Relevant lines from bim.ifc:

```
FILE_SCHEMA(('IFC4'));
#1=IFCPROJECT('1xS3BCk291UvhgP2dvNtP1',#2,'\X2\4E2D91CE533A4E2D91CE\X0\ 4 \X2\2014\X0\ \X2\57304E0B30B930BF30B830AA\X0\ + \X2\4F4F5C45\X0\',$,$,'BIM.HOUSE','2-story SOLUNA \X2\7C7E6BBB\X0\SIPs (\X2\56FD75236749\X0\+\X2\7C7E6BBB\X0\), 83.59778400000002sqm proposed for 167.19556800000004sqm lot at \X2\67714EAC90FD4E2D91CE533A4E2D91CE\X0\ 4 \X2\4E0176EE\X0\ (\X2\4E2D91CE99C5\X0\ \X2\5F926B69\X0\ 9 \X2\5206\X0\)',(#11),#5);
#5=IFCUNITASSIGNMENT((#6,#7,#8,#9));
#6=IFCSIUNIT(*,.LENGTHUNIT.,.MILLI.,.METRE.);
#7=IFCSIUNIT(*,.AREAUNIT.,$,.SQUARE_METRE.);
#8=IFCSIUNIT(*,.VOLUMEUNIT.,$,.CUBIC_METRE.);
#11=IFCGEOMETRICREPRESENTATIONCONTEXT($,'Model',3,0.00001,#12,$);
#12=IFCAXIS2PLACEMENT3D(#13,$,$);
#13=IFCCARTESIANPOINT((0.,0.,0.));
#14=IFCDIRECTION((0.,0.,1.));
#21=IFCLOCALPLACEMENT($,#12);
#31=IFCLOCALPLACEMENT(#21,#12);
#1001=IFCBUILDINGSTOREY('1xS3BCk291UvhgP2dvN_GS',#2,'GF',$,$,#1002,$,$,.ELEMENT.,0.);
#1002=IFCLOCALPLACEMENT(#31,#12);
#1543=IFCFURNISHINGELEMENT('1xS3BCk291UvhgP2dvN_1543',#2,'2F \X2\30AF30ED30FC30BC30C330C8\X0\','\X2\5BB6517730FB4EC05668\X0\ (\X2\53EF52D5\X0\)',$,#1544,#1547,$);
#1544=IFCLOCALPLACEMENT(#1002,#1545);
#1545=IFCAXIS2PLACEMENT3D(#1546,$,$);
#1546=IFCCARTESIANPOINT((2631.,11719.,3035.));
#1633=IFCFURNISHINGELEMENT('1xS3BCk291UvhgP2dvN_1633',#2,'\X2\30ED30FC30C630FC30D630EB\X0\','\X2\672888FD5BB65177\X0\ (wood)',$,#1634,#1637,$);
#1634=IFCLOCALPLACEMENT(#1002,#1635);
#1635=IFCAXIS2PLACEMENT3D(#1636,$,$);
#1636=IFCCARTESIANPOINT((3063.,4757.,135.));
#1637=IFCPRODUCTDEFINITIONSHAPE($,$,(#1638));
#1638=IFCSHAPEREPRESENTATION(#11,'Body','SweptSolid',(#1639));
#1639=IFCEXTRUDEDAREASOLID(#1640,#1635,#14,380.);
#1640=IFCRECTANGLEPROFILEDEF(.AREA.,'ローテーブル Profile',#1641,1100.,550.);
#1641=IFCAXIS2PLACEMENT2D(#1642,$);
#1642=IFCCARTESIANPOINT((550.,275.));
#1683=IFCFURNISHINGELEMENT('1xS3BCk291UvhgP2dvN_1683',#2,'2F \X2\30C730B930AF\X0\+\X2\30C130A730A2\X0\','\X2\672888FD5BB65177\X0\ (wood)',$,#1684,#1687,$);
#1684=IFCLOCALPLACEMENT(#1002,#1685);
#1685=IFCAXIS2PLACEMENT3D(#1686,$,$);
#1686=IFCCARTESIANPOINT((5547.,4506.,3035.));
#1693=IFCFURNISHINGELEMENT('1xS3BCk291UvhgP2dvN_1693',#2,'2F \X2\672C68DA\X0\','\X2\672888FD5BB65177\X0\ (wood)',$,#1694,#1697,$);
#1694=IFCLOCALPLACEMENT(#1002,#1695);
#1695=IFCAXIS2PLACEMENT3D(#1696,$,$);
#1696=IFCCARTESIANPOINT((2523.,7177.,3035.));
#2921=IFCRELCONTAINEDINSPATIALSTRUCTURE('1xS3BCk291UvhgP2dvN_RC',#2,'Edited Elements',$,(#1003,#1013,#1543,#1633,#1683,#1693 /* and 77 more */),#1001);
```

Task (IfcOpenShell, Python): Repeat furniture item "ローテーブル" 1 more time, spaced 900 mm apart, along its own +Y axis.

```python
import ifcopenshell
import ifcopenshell.api.geometry
import ifcopenshell.api.root
import ifcopenshell.util.element
import ifcopenshell.util.placement
import ifcopenshell.util.unit

model = ifcopenshell.open("bim.ifc")
unit_scale = ifcopenshell.util.unit.calculate_unit_scale(model)


def reuse_history(source, copy):
    """copy_class also copies each property set's owner history, people and application; keep the originals."""
    for rel in copy.IsDefinedBy:
        if rel.is_a("IfcRelDefinesByProperties") and (history := rel.RelatingPropertyDefinition.OwnerHistory):
            rel.RelatingPropertyDefinition.OwnerHistory = source.OwnerHistory
            ifcopenshell.util.element.remove_deep2(model, history)


source = model.by_guid("1xS3BCk291UvhgP2dvN_1633")
base = ifcopenshell.util.placement.get_local_placement(source.ObjectPlacement)
step = base[:3, 1] * 0.9 / unit_scale

for i in range(1, 2):
    copy = ifcopenshell.api.root.copy_class(model, product=source)
    copy.Representation = ifcopenshell.util.element.copy_deep(
        model, source.Representation, exclude=["IfcGeometricRepresentationContext", "IfcRepresentationMap"]
    )
    reuse_history(source, copy)
    matrix = base.copy()
    matrix[:3, 3] += i * step
    print("added at", matrix[:3, 3].round(3) + 0.0)
    ifcopenshell.api.geometry.edit_object_placement(model, product=copy, matrix=matrix, is_si=False)

model.write("bim_edited.ifc")
```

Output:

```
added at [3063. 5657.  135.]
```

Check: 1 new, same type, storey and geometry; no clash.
